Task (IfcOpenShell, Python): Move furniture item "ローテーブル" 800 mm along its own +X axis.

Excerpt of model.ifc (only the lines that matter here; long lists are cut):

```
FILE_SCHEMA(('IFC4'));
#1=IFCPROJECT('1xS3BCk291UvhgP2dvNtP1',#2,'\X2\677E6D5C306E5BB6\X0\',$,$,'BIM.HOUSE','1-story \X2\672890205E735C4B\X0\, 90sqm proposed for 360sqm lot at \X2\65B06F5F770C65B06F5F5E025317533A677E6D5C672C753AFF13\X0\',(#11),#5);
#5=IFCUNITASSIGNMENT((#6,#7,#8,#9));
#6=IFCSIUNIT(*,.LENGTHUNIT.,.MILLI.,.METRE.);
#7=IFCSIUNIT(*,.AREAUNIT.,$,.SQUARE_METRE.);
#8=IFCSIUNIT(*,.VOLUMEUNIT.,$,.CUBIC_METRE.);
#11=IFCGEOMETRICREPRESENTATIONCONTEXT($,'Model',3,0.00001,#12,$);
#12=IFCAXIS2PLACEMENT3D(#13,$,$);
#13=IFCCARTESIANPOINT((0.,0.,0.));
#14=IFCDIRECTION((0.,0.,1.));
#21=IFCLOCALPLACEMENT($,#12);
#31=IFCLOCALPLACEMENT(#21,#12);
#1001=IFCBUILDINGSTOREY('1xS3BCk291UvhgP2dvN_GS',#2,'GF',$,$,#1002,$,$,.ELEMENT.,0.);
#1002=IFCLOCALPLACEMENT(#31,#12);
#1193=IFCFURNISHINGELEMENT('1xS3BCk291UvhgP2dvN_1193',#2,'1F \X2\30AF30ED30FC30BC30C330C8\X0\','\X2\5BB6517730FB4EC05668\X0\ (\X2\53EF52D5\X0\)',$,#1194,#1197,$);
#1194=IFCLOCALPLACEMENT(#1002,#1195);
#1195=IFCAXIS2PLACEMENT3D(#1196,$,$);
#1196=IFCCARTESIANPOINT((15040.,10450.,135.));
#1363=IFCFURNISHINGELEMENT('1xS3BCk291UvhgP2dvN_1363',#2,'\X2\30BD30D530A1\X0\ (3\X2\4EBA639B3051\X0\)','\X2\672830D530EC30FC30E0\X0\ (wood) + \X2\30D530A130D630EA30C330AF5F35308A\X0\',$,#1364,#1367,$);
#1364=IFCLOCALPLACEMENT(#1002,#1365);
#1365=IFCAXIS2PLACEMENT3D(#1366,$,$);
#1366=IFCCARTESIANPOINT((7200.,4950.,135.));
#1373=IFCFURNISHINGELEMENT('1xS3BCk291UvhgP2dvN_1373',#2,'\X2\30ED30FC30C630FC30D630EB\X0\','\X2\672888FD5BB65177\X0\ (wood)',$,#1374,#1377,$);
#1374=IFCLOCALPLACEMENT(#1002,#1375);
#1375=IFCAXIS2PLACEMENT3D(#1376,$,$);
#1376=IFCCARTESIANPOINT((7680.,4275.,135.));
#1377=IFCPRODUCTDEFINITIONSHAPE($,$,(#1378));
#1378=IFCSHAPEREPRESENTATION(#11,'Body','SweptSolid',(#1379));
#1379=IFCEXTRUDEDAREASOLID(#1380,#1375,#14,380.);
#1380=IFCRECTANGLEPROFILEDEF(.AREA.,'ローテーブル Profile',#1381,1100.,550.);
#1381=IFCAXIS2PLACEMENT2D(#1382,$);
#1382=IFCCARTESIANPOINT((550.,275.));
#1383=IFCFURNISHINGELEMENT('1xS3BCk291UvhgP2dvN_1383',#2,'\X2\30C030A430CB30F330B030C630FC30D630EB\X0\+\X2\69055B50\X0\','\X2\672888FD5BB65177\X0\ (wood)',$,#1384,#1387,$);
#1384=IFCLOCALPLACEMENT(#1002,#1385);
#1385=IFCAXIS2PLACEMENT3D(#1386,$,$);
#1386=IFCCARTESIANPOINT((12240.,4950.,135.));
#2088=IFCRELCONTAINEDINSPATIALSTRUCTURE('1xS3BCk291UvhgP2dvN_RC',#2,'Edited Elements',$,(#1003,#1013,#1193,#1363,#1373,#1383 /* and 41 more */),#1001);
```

```python
import ifcopenshell
import ifcopenshell.api.geometry
import ifcopenshell.util.placement

model = ifcopenshell.open("model.ifc")

item = model.by_guid("1xS3BCk291UvhgP2dvN_1373")
matrix = ifcopenshell.util.placement.get_local_placement(item.ObjectPlacement)
matrix[:3, 3] += matrix[:3, 0] * 800.0
ifcopenshell.api.geometry.edit_object_placement(model, product=item, matrix=matrix, is_si=False)

print(ifcopenshell.util.placement.get_local_placement(item.ObjectPlacement).round(3) + 0.0)

model.write("model_rev.ifc")
```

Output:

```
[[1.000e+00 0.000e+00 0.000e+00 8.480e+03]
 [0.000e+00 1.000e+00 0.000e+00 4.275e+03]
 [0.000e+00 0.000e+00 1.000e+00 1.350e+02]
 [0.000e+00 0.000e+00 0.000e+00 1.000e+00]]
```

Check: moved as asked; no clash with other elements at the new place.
